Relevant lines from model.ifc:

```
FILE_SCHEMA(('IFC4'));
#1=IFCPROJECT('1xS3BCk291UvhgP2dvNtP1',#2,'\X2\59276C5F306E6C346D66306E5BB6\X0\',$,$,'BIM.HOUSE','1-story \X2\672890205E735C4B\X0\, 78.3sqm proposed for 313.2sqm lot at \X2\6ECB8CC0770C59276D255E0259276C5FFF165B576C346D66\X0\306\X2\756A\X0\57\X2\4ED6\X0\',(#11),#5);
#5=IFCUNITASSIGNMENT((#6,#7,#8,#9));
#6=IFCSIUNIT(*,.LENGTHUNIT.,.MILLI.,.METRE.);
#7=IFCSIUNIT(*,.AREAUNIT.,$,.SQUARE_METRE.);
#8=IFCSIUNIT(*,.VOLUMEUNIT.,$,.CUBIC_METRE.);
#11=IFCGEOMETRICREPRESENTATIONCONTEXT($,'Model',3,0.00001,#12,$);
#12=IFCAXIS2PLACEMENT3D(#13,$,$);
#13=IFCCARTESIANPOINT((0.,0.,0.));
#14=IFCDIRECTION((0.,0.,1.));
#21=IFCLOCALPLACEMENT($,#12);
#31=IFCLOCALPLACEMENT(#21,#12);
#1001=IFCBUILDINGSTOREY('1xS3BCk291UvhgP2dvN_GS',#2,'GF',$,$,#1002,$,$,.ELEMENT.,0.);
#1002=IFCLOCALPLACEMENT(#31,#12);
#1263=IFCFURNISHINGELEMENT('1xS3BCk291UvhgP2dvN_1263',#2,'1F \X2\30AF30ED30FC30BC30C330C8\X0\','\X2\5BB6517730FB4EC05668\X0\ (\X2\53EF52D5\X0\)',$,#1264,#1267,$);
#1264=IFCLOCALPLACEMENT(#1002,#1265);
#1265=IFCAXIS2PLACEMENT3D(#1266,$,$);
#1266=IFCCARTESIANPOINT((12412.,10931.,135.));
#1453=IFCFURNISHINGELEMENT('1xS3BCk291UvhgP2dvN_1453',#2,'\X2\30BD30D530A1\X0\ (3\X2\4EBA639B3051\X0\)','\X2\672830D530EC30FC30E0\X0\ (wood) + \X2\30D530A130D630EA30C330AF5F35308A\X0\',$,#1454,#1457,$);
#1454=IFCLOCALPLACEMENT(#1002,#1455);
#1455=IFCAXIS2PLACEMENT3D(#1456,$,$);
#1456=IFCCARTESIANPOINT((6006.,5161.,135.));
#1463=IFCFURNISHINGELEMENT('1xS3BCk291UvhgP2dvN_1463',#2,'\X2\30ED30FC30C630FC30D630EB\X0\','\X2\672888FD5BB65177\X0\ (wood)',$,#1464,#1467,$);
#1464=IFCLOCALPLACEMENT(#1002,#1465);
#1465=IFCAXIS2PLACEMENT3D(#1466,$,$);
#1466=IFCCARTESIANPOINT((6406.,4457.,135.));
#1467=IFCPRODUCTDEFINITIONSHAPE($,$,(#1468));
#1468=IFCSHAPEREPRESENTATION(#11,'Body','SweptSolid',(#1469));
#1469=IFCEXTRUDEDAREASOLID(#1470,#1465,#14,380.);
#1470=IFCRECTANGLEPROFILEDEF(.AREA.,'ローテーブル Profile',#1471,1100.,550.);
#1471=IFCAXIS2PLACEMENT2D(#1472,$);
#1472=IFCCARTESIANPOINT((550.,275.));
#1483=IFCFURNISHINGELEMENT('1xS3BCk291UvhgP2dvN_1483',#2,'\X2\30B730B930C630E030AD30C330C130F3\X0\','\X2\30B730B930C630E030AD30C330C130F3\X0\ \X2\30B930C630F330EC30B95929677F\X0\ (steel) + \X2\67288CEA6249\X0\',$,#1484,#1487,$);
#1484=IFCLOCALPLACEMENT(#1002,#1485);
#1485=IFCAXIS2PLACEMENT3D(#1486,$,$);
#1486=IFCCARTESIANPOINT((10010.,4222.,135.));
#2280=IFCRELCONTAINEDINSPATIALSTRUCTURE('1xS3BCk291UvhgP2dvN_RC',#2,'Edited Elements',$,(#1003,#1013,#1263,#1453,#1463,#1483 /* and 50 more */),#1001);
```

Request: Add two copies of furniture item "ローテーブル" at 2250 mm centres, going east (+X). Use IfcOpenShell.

```python
import numpy as np
import ifcopenshell
import ifcopenshell.api.geometry
import ifcopenshell.api.root
import ifcopenshell.util.element
import ifcopenshell.util.placement

model = ifcopenshell.open("model.ifc")


def reuse_history(source, copy):
    """copy_class also copies each property set's owner history, people and application; keep the originals."""
    for rel in copy.IsDefinedBy:
        if rel.is_a("IfcRelDefinesByProperties") and (history := rel.RelatingPropertyDefinition.OwnerHistory):
            rel.RelatingPropertyDefinition.OwnerHistory = source.OwnerHistory
            ifcopenshell.util.element.remove_deep2(model, history)


source = model.by_id(1463)
base = ifcopenshell.util.placement.get_local_placement(source.ObjectPlacement)
step = np.array([1.0, 0.0, 0.0]) * 2250.0

for i in range(1, 3):
    copy = ifcopenshell.api.root.copy_class(model, product=source)
    copy.Representation = ifcopenshell.util.element.copy_deep(
        model, source.Representation, exclude=["IfcGeometricRepresentationContext", "IfcRepresentationMap"]
    )
    reuse_history(source, copy)
    matrix = base.copy()
    matrix[:3, 3] += i * step
    print("added at", matrix[:3, 3].round(3) + 0.0)
    ifcopenshell.api.geometry.edit_object_placement(model, product=copy, matrix=matrix, is_si=False)

model.write("model-out.ifc")
```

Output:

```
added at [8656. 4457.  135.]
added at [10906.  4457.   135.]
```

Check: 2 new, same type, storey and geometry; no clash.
